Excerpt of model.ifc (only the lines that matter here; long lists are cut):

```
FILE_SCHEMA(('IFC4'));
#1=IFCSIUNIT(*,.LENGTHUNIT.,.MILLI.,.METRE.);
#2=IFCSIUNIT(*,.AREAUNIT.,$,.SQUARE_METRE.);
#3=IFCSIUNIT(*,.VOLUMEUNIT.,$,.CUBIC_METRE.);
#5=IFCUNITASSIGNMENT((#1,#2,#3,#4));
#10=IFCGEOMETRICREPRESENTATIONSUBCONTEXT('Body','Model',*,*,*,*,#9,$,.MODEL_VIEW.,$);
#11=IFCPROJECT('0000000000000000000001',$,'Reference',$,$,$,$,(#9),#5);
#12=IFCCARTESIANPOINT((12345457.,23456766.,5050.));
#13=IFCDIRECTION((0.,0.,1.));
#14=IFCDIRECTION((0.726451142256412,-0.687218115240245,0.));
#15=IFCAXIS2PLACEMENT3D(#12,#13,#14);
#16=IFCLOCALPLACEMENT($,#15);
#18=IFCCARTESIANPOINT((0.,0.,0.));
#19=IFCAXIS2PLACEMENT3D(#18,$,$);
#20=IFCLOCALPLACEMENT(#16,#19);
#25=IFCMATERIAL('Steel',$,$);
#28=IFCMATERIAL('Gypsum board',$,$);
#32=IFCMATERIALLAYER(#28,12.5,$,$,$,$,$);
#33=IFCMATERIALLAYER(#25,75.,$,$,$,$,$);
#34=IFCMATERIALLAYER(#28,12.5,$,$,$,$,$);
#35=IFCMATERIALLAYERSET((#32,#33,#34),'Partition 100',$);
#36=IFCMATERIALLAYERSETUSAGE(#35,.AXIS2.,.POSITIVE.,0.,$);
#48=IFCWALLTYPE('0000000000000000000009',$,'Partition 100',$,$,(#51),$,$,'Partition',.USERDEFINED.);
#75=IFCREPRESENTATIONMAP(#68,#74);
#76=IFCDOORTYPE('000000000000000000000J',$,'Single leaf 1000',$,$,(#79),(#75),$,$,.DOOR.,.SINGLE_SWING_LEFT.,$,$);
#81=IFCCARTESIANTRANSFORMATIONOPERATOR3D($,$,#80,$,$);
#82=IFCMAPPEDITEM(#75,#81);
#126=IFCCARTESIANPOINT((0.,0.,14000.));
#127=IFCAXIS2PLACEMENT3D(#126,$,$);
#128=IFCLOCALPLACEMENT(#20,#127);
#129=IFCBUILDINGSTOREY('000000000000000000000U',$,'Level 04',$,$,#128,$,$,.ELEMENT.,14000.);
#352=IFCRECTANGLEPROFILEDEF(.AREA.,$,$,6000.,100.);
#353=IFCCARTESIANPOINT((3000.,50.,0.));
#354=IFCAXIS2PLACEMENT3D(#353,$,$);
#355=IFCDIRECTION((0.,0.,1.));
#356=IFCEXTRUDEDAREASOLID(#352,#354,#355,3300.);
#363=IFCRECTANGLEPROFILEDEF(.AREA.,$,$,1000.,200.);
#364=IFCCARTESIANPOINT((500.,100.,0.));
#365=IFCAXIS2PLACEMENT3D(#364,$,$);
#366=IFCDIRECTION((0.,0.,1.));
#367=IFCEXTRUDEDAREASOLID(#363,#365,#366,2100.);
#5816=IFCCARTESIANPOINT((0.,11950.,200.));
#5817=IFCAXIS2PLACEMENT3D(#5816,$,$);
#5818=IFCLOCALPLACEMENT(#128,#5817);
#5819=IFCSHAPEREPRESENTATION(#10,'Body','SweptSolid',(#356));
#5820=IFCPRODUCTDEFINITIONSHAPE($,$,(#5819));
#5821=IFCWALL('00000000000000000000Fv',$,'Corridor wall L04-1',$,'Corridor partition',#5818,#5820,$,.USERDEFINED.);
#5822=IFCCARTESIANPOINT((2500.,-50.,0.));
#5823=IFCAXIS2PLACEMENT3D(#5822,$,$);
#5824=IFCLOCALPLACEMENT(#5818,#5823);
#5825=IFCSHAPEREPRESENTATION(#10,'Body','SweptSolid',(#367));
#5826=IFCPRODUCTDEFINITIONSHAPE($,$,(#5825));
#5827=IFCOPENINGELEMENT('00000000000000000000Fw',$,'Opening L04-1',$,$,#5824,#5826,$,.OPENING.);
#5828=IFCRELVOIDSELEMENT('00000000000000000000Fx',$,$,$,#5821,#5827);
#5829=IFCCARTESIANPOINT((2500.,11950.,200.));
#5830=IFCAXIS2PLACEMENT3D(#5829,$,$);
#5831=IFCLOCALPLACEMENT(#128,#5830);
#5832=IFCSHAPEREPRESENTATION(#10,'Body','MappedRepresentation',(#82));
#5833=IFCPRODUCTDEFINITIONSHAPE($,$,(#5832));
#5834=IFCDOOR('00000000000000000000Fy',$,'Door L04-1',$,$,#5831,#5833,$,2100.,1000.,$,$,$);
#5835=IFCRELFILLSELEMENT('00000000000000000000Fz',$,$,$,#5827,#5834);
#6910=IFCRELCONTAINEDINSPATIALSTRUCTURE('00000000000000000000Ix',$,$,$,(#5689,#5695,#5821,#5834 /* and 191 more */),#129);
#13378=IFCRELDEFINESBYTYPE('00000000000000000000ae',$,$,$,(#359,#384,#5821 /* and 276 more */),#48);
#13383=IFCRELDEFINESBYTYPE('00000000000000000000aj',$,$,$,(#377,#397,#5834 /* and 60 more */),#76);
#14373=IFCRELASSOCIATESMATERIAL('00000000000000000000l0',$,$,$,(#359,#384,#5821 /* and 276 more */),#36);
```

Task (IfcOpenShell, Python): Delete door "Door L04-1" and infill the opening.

```python
import ifcopenshell
import ifcopenshell.api.feature
import ifcopenshell.api.root
import ifcopenshell.geom
import ifcopenshell.util.shape

model = ifcopenshell.open("model.ifc")
settings = ifcopenshell.geom.settings()


def volume(element):
    """Net volume in cubic metres, openings subtracted."""
    shape = ifcopenshell.geom.create_shape(settings, element)
    return ifcopenshell.util.shape.get_volume(shape.geometry)


door = model.by_guid("00000000000000000000Fy")
opening = door.FillsVoids[0].RelatingOpeningElement
wall = opening.VoidsElements[0].RelatingBuildingElement
before = volume(wall)

ifcopenshell.api.root.remove_product(model, product=door)
ifcopenshell.api.feature.remove_feature(model, feature=opening)

after = volume(wall)

print(f"wall volume {before:.3f} -> {after:.3f} m3")

model.write("model_v2.ifc")
```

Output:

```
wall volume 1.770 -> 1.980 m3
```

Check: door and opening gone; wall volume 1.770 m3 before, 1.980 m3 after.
